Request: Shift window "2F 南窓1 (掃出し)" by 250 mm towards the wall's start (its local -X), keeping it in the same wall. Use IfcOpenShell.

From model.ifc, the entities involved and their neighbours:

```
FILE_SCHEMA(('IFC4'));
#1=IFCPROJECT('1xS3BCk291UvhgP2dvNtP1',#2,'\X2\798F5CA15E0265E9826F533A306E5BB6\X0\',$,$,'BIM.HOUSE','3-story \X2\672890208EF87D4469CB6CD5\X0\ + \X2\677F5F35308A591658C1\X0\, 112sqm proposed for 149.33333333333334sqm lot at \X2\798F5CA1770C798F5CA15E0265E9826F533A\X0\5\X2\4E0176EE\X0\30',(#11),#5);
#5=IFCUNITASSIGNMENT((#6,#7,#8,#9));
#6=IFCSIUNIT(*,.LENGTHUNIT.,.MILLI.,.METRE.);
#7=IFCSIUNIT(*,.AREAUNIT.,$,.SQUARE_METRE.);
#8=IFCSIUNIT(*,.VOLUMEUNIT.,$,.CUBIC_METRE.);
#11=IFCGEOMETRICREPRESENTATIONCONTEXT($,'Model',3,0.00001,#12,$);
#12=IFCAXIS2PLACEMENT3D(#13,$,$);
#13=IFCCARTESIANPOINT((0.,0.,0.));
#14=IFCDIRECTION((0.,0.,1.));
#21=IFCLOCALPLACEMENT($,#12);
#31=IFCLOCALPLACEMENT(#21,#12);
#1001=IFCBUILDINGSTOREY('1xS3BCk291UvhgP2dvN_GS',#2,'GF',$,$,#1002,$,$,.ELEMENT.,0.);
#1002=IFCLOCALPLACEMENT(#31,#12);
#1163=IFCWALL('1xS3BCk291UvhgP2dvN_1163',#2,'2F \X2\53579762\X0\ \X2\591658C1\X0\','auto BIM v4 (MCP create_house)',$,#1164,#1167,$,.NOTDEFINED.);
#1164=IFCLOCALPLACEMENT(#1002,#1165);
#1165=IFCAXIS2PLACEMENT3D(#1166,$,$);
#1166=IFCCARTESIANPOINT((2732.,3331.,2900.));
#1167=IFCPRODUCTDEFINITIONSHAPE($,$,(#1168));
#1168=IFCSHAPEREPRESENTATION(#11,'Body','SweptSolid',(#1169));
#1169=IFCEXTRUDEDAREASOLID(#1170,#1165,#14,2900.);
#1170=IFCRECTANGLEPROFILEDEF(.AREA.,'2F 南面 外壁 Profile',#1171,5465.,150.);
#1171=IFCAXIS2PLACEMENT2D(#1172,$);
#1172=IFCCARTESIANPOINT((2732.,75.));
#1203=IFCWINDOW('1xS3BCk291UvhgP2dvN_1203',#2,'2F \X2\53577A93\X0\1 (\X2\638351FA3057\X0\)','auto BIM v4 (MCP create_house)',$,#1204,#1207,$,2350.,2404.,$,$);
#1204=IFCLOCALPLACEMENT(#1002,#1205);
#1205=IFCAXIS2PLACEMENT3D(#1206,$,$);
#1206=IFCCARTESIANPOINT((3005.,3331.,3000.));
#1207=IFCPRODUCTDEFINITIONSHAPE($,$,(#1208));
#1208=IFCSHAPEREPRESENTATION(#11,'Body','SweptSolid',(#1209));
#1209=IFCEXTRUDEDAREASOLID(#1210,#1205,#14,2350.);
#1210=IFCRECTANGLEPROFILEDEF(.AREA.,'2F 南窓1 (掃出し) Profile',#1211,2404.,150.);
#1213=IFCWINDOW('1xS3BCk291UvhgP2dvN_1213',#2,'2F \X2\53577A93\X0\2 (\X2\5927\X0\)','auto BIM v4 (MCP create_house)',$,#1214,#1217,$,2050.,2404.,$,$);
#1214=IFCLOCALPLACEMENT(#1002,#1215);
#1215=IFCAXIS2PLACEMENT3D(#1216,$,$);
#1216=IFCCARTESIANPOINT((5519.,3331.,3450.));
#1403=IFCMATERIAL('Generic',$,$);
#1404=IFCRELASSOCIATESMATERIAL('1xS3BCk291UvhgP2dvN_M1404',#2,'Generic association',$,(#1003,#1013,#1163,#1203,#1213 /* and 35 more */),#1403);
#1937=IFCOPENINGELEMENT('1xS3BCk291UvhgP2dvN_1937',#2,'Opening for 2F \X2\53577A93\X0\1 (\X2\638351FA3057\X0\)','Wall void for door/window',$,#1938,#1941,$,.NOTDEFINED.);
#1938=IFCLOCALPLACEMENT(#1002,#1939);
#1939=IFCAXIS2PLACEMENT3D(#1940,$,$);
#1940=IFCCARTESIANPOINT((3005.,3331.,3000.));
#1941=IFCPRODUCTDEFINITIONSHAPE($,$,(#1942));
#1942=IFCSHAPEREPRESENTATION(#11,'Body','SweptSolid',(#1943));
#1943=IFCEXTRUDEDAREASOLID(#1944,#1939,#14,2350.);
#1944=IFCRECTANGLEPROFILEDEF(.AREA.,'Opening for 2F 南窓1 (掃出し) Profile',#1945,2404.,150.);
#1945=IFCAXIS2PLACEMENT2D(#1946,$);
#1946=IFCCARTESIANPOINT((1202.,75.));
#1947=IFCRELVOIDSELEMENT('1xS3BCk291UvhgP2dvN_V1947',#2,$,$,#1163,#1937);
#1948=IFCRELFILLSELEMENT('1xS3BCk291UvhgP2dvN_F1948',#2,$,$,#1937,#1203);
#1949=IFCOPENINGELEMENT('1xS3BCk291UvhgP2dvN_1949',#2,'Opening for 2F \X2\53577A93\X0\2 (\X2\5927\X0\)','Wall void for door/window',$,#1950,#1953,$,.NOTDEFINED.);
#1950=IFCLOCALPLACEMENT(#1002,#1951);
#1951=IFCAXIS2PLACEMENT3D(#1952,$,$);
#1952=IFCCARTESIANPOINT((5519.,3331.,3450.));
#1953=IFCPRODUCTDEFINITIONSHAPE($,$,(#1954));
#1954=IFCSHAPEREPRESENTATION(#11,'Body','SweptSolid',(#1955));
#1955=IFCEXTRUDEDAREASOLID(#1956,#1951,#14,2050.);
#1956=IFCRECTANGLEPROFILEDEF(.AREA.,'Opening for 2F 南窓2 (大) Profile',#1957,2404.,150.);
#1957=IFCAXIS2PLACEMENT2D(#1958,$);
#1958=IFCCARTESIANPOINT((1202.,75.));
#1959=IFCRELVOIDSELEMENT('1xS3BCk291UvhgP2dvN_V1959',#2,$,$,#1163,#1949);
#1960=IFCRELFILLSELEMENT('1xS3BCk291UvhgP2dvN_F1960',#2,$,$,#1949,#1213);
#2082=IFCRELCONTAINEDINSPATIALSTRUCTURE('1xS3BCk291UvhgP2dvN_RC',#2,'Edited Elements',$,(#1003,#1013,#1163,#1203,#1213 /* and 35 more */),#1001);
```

```python
import ifcopenshell
import ifcopenshell.api.geometry
import ifcopenshell.util.placement

model = ifcopenshell.open("model.ifc")

window = model.by_id(1203)
opening = window.FillsVoids[0].RelatingOpeningElement
wall = opening.VoidsElements[0].RelatingBuildingElement

wall_matrix = ifcopenshell.util.placement.get_local_placement(wall.ObjectPlacement)
shift = wall_matrix[:3, 0] * -250.0
before = ifcopenshell.util.placement.get_local_placement(window.ObjectPlacement)[:3, 3].copy()

# The window is not placed relative to its opening, so move both.
for product in (opening, window):
    matrix = ifcopenshell.util.placement.get_local_placement(product.ObjectPlacement)
    matrix[:3, 3] += shift
    ifcopenshell.api.geometry.edit_object_placement(model, product=product, matrix=matrix, is_si=False)

after = ifcopenshell.util.placement.get_local_placement(window.ObjectPlacement)[:3, 3]
print("window moved by", (after - before).round(3) + 0.0)

model.write("model_rev.ifc")
```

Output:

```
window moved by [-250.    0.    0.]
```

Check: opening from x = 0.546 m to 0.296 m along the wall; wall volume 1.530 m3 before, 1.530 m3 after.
